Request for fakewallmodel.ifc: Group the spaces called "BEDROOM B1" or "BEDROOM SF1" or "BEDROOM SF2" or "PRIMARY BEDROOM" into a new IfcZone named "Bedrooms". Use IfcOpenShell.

First a look at what the model holds.

```python
import ifcopenshell

model = ifcopenshell.open("fakewallmodel.ifc")
print(model.schema)
seen = {}
for space in model.by_type("IfcSpace"):
    seen[space.LongName] = seen.get(space.LongName, 0) + 1
for name, count in sorted(seen.items(), key=str):
    print(count, "x", name)
print("zones:", [z.Name for z in model.by_type("IfcZone")][:20])
```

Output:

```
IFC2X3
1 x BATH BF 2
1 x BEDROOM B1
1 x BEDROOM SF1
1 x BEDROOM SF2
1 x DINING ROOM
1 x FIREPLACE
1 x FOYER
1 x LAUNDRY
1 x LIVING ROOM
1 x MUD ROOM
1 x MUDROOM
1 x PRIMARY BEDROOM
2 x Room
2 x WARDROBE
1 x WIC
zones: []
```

```python
import ifcopenshell
import ifcopenshell.api.group
import ifcopenshell.api.root

model = ifcopenshell.open("fakewallmodel.ifc")

names = {"BEDROOM B1", "BEDROOM SF1", "BEDROOM SF2", "PRIMARY BEDROOM"}
spaces = [s for s in model.by_type("IfcSpace") if s.LongName in names]

zone = ifcopenshell.api.root.create_entity(model, ifc_class="IfcZone", name="Bedrooms")
ifcopenshell.api.group.assign_group(model, products=spaces, group=zone)
print(len(spaces), "spaces in", zone.Name)

model.write("fakewallmodel_v2.ifc")
```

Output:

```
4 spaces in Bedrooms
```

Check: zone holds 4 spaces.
